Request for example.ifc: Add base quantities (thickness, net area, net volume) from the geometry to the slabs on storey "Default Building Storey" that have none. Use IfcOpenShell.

First a look at what the model holds.

```python
import ifcopenshell
import ifcopenshell.util.element
import ifcopenshell.util.unit

model = ifcopenshell.open("example.ifc")
print(model.schema)
for unit_type in ("LENGTHUNIT", "AREAUNIT", "VOLUMEUNIT"):
    print(unit_type, ifcopenshell.util.unit.calculate_unit_scale(model, unit_type))
storey = next(s for s in model.by_type("IfcBuildingStorey") if s.Name == "Default Building Storey")
slabs = [e for e in ifcopenshell.util.element.get_decomposition(storey) if e.is_a("IfcSlab")]
for e in sorted(slabs, key=lambda e: e.id()):
    print(e.id(), e.is_a(), e.Name, list(ifcopenshell.util.element.get_psets(e, qtos_only=True)), sep=" | ")
```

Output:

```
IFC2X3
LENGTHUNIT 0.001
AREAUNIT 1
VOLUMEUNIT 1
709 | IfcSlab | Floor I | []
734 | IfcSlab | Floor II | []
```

```python
import ifcopenshell
import ifcopenshell.api.pset
import ifcopenshell.geom
import ifcopenshell.util.element
import ifcopenshell.util.shape
import ifcopenshell.util.unit

model = ifcopenshell.open("example.ifc")
unit_scale = ifcopenshell.util.unit.calculate_unit_scale(model)
area_scale = ifcopenshell.util.unit.calculate_unit_scale(model, "AREAUNIT")
volume_scale = ifcopenshell.util.unit.calculate_unit_scale(model, "VOLUMEUNIT")
settings = ifcopenshell.geom.settings()

storey = next(s for s in model.by_type("IfcBuildingStorey") if s.Name == "Default Building Storey")
slabs = [e for e in ifcopenshell.util.element.get_decomposition(storey) if e.is_a("IfcSlab")]

for e in sorted(slabs, key=lambda e: e.id()):
    if ifcopenshell.util.element.get_psets(e, qtos_only=True, should_inherit=False):
        continue
    # Geometry comes back in metres, in the element's own axes.
    shape = ifcopenshell.geom.create_shape(settings, e)
    values = {
        "Width": ifcopenshell.util.shape.get_z(shape.geometry) / unit_scale,
        "NetArea": ifcopenshell.util.shape.get_footprint_area(shape.geometry) / area_scale,
        "NetVolume": ifcopenshell.util.shape.get_volume(shape.geometry) / volume_scale,
    }
    qto = ifcopenshell.api.pset.add_qto(model, product=e, name="BaseQuantities")
    ifcopenshell.api.pset.edit_qto(model, qto=qto, properties=values)
    print(e.id(), {k: round(v, 3) for k, v in values.items()})

model.write("example_v2.ifc")
```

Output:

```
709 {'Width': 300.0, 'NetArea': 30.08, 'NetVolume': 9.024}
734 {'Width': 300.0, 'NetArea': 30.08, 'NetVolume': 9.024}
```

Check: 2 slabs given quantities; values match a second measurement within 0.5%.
